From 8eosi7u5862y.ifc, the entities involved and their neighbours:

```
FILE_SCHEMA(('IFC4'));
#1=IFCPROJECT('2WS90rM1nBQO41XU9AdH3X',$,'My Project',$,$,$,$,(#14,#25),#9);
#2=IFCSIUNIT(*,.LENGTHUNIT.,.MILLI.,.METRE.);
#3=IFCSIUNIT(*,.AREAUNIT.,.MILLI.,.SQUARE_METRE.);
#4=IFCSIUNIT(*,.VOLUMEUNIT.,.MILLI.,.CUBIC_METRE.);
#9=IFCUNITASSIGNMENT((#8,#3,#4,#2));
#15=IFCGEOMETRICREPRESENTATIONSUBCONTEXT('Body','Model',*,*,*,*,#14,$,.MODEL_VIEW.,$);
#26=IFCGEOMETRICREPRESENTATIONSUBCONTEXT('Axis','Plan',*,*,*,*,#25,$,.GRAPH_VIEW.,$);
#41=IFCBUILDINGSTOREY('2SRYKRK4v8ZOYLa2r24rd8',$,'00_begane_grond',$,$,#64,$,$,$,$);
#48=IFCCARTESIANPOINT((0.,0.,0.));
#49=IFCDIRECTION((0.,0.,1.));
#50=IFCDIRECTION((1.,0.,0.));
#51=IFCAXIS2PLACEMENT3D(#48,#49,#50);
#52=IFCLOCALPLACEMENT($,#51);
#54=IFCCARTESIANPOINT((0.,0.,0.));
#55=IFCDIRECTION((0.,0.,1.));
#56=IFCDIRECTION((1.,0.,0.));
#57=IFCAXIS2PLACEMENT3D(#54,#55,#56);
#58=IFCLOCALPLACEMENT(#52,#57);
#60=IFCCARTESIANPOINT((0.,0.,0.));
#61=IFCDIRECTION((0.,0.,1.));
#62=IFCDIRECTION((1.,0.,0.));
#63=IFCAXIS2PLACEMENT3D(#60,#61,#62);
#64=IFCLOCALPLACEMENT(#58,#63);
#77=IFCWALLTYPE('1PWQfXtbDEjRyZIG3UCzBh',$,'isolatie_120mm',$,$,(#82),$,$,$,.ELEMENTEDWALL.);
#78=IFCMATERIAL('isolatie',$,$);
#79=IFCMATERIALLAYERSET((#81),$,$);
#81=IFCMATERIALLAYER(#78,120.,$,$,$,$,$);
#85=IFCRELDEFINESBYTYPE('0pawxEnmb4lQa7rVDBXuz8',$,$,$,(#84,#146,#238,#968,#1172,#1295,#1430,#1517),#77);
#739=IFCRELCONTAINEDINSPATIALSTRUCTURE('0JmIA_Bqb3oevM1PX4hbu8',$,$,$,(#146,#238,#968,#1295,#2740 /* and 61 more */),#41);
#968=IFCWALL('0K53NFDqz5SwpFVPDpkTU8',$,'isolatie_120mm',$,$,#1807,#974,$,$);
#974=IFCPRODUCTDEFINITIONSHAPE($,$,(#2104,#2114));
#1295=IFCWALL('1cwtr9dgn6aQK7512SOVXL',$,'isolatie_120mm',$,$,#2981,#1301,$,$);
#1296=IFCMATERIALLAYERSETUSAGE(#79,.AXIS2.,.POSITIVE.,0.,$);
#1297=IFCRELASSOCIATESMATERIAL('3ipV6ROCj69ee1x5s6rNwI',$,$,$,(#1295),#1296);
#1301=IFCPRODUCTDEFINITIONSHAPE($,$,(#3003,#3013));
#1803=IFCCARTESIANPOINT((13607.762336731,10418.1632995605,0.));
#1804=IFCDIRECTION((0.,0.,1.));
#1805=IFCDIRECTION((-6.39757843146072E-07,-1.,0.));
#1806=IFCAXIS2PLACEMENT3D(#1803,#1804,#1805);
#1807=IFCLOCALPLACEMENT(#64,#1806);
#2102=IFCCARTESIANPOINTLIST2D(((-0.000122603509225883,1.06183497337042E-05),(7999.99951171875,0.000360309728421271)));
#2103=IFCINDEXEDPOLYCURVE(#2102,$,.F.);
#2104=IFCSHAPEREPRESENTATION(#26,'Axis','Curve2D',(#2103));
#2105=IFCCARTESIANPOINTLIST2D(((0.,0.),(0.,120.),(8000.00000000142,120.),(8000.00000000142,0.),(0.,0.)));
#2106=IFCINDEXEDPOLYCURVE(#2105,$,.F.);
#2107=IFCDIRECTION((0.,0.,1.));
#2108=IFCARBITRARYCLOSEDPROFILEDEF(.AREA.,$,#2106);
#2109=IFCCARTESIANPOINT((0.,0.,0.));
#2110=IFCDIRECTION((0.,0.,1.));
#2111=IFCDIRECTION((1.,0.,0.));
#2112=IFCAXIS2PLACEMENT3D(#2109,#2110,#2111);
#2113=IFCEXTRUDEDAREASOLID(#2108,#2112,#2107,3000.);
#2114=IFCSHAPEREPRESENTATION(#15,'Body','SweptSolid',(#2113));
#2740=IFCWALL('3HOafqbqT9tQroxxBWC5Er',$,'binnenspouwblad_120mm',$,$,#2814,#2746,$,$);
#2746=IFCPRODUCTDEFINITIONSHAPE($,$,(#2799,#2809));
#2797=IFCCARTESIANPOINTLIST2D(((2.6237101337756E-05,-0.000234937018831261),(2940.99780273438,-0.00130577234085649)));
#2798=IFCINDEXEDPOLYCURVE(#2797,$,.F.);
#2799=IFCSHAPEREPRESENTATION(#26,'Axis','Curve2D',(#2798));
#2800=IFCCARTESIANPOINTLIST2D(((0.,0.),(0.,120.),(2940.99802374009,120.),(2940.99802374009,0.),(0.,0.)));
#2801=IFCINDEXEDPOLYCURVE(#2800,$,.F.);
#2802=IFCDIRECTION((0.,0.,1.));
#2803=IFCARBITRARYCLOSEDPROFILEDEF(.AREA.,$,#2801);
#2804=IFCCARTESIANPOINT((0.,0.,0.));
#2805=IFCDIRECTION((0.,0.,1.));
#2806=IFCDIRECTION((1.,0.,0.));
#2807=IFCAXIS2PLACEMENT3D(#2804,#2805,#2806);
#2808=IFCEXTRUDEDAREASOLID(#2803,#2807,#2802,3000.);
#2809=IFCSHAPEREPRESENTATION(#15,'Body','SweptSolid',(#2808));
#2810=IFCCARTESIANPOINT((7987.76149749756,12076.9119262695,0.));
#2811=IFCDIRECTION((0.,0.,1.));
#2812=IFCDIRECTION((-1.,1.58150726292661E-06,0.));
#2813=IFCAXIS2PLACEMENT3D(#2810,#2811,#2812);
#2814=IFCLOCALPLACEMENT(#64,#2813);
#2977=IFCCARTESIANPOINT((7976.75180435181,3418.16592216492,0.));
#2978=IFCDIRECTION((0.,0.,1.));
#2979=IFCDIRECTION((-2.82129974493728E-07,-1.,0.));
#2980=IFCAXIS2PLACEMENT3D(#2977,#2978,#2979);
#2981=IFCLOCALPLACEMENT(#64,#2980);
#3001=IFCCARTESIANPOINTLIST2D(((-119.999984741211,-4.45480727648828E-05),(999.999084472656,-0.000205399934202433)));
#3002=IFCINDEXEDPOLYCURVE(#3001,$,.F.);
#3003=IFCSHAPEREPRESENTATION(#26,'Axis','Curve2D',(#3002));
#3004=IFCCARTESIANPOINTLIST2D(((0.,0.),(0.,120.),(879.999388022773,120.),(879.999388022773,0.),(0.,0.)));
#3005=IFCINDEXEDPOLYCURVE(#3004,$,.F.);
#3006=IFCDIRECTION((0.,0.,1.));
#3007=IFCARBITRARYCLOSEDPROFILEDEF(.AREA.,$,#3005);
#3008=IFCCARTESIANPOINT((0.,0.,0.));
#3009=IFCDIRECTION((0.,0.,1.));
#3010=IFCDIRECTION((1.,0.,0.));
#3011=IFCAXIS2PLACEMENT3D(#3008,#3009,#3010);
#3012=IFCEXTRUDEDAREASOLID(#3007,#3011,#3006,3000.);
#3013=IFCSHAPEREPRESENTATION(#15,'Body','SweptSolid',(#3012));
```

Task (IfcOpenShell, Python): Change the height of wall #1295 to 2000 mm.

```python
import ifcopenshell
import ifcopenshell.geom
import ifcopenshell.util.representation
import ifcopenshell.util.shape
import ifcopenshell.util.unit

model = ifcopenshell.open("8eosi7u5862y.ifc")
unit_scale = ifcopenshell.util.unit.calculate_unit_scale(model)
settings = ifcopenshell.geom.settings()


def volume(element):
    """Net volume in cubic metres, openings subtracted."""
    shape = ifcopenshell.geom.create_shape(settings, element)
    return ifcopenshell.util.shape.get_volume(shape.geometry)


wall = model.by_guid("1cwtr9dgn6aQK7512SOVXL")
before = volume(wall)

body = ifcopenshell.util.representation.get_representation(wall, "Model", "Body")
solid = body.Items[0]
old_height = solid.Depth
solid.Depth = 2 / unit_scale
after = volume(wall)

print(f"height {old_height:g} -> {solid.Depth:g}, volume {before:.3f} -> {after:.3f} m3")

model.write("8eosi7u5862y_rev.ifc")
```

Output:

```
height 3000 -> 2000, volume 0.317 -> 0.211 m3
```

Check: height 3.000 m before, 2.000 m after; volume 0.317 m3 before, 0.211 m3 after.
